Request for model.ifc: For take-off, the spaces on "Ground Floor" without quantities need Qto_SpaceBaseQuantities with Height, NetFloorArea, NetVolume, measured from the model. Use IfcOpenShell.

First a look at what the model holds.

```python
import ifcopenshell
import ifcopenshell.util.element
import ifcopenshell.util.unit

model = ifcopenshell.open("model.ifc")
print(model.schema)
for unit_type in ("LENGTHUNIT", "AREAUNIT", "VOLUMEUNIT"):
    print(unit_type, ifcopenshell.util.unit.calculate_unit_scale(model, unit_type))
storey = next(s for s in model.by_type("IfcBuildingStorey") if s.Name == "Ground Floor")
spaces = [e for e in ifcopenshell.util.element.get_decomposition(storey) if e.is_a("IfcSpace")]
for e in sorted(spaces, key=lambda e: e.id()):
    print(e.id(), e.is_a(), e.Name, list(ifcopenshell.util.element.get_psets(e, qtos_only=True)), sep=" | ")
```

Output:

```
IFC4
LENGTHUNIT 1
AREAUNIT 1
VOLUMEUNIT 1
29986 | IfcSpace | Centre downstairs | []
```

```python
import ifcopenshell
import ifcopenshell.api.pset
import ifcopenshell.geom
import ifcopenshell.util.element
import ifcopenshell.util.shape
import ifcopenshell.util.unit

model = ifcopenshell.open("model.ifc")
unit_scale = ifcopenshell.util.unit.calculate_unit_scale(model)
area_scale = ifcopenshell.util.unit.calculate_unit_scale(model, "AREAUNIT")
volume_scale = ifcopenshell.util.unit.calculate_unit_scale(model, "VOLUMEUNIT")
settings = ifcopenshell.geom.settings()

storey = next(s for s in model.by_type("IfcBuildingStorey") if s.Name == "Ground Floor")
spaces = [e for e in ifcopenshell.util.element.get_decomposition(storey) if e.is_a("IfcSpace")]

for e in sorted(spaces, key=lambda e: e.id()):
    if ifcopenshell.util.element.get_psets(e, qtos_only=True, should_inherit=False):
        continue
    # Geometry comes back in metres, in the element's own axes.
    shape = ifcopenshell.geom.create_shape(settings, e)
    values = {
        "Height": ifcopenshell.util.shape.get_z(shape.geometry) / unit_scale,
        "NetFloorArea": ifcopenshell.util.shape.get_footprint_area(shape.geometry) / area_scale,
        "NetVolume": ifcopenshell.util.shape.get_volume(shape.geometry) / volume_scale,
    }
    qto = ifcopenshell.api.pset.add_qto(model, product=e, name="Qto_SpaceBaseQuantities")
    ifcopenshell.api.pset.edit_qto(model, qto=qto, properties=values)
    print(e.id(), {k: round(v, 3) for k, v in values.items()})

model.write("model_edited.ifc")
```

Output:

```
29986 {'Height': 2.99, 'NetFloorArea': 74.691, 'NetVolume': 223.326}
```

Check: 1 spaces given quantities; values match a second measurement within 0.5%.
